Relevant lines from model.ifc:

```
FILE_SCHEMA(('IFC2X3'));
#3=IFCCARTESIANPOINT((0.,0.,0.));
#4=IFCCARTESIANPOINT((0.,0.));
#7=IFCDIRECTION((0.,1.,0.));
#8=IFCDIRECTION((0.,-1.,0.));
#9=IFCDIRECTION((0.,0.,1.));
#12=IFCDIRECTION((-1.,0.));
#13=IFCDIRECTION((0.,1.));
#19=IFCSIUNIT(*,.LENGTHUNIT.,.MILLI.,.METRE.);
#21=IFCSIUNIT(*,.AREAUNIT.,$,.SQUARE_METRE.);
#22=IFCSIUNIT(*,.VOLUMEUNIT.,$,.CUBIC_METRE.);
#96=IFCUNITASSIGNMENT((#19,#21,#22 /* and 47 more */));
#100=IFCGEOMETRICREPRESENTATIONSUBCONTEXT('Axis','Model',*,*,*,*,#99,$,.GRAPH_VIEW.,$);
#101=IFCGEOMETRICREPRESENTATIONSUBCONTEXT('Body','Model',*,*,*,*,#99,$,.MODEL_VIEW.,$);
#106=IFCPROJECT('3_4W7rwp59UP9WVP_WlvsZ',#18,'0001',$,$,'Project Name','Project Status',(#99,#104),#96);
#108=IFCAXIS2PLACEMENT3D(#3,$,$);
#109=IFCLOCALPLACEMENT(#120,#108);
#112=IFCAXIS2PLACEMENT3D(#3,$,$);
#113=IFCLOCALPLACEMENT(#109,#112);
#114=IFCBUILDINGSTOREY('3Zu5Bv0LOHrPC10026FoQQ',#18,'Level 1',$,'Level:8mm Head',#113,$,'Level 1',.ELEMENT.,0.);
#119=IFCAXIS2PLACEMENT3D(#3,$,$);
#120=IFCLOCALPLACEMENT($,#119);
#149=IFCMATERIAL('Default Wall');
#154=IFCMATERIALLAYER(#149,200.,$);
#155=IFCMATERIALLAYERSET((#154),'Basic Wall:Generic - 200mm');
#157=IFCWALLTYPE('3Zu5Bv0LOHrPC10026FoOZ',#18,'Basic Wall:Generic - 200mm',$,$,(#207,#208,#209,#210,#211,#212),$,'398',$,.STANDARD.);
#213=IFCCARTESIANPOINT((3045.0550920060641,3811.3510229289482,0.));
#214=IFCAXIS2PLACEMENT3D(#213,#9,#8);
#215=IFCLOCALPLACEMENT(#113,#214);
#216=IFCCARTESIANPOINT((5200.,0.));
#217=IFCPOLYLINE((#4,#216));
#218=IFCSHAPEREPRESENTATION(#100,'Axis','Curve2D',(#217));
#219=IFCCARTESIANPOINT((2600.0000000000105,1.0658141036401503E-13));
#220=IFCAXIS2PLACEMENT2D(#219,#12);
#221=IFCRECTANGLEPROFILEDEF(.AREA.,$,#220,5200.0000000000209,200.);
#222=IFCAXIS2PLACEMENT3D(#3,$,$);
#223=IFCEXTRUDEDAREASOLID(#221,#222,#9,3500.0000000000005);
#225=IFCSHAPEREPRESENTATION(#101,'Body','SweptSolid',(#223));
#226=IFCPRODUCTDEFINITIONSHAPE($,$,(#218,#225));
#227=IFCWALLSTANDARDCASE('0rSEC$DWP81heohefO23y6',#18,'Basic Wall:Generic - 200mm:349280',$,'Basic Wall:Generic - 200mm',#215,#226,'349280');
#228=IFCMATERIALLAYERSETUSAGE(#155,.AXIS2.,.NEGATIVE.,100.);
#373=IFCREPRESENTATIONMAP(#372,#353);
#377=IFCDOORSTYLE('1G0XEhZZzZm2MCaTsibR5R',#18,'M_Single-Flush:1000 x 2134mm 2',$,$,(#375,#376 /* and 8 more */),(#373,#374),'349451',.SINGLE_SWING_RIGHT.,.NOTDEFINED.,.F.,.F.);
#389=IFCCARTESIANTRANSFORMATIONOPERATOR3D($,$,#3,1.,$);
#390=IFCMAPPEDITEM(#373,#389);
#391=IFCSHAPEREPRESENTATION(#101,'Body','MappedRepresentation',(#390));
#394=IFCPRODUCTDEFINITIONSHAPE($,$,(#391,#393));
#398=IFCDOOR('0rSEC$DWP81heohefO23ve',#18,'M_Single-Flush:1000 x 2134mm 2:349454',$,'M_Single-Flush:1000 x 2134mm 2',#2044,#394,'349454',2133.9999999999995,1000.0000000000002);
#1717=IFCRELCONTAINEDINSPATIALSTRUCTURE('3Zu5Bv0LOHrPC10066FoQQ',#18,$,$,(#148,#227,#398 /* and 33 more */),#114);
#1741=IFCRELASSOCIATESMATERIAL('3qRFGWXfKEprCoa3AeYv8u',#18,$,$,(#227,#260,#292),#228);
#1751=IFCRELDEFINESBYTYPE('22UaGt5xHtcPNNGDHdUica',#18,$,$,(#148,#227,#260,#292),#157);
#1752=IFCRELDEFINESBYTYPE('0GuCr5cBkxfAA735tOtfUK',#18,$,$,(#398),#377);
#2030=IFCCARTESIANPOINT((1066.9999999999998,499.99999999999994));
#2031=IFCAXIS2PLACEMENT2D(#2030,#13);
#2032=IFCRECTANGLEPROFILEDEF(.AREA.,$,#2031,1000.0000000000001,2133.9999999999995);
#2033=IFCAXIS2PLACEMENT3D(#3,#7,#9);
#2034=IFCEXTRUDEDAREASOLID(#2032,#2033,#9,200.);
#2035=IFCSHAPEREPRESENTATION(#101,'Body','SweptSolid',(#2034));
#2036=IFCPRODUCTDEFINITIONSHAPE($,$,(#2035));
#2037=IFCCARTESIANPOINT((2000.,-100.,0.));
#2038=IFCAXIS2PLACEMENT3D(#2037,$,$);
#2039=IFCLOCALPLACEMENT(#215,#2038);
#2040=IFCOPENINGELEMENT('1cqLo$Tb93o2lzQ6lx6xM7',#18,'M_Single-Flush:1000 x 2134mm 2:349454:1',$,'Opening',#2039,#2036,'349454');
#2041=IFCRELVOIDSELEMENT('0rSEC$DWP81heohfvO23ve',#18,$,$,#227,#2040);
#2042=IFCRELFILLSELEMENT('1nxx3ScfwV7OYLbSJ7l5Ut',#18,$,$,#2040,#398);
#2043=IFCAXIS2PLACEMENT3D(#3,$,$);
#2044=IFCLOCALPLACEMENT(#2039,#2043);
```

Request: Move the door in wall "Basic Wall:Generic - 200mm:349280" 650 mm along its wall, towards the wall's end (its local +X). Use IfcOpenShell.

```python
import ifcopenshell
import ifcopenshell.api.geometry
import ifcopenshell.util.placement
import ifcopenshell.util.unit

model = ifcopenshell.open("model.ifc")
unit_scale = ifcopenshell.util.unit.calculate_unit_scale(model)

door = model.by_guid("0rSEC$DWP81heohefO23ve")
opening = door.FillsVoids[0].RelatingOpeningElement
wall = opening.VoidsElements[0].RelatingBuildingElement

wall_matrix = ifcopenshell.util.placement.get_local_placement(wall.ObjectPlacement)
shift = wall_matrix[:3, 0] * 0.65 / unit_scale
before = ifcopenshell.util.placement.get_local_placement(door.ObjectPlacement)[:3, 3].copy()

# The door is placed relative to its opening, so it follows when the opening moves.
matrix = ifcopenshell.util.placement.get_local_placement(opening.ObjectPlacement)
matrix[:3, 3] += shift
ifcopenshell.api.geometry.edit_object_placement(
    model, product=opening, matrix=matrix, is_si=False, should_transform_children=True
)

after = ifcopenshell.util.placement.get_local_placement(door.ObjectPlacement)[:3, 3]
print("door moved by", (after - before).round(3) + 0.0)

model.write("model-out.ifc")
```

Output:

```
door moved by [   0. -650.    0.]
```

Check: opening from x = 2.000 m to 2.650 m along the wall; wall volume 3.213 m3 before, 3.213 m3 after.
